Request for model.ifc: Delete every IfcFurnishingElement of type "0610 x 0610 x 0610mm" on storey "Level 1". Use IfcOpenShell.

First a look at what the model holds.

```python
import ifcopenshell
import ifcopenshell.util.element

model = ifcopenshell.open("model.ifc")
print(model.schema)
storey = next(s for s in model.by_type("IfcBuildingStorey") if s.Name == "Level 1")
furniture = [e for e in ifcopenshell.util.element.get_decomposition(storey) if e.is_a("IfcFurnishingElement")]
seen = {}
for e in furniture:
    element_type = ifcopenshell.util.element.get_type(e)
    name = element_type.Name if element_type not in (None, e) else None
    seen[name] = seen.get(name, 0) + 1
for name, count in sorted(seen.items(), key=str):
    print(count, "x", name)
```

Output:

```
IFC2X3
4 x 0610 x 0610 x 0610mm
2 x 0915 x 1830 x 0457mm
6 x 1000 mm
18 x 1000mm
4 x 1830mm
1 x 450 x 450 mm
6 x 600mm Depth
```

```python
import ifcopenshell
import ifcopenshell.api.root
import ifcopenshell.util.element

model = ifcopenshell.open("model.ifc")

storey = next(s for s in model.by_type("IfcBuildingStorey") if s.Name == "Level 1")
furniture = [e for e in ifcopenshell.util.element.get_decomposition(storey) if e.is_a("IfcFurnishingElement")]
targets = [e for e in furniture if (t := ifcopenshell.util.element.get_type(e)) not in (None, e) and t.Name == "0610 x 0610 x 0610mm"]

for e in targets:
    ifcopenshell.api.root.remove_product(model, product=e)
print(len(targets), "removed")

model.write("model_rev.ifc")
```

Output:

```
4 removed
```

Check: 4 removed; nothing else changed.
